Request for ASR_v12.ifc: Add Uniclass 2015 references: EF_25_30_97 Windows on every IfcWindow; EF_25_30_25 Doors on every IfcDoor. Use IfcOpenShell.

First a look at what the model holds.

```python
import ifcopenshell

model = ifcopenshell.open("ASR_v12.ifc")
print(model.schema)
print("classifications:", [c.Name for c in model.by_type("IfcClassification")])
for ifc_class in ("IfcDoor", "IfcRoof", "IfcStair", "IfcWall", "IfcWindow"):
    print(ifc_class, len(model.by_type(ifc_class)))
```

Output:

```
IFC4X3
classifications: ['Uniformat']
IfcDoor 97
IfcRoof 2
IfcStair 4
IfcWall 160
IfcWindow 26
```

```python
import ifcopenshell
import ifcopenshell.api.classification

model = ifcopenshell.open("ASR_v12.ifc")

system = ifcopenshell.api.classification.add_classification(model, classification="Uniclass 2015")

codes = {
    "IfcWindow": ("EF_25_30_97", "Windows"),
    "IfcDoor": ("EF_25_30_25", "Doors"),
}
for ifc_class, (code, name) in codes.items():
    products = model.by_type(ifc_class)
    ifcopenshell.api.classification.add_reference(
        model, products=products, classification=system, identification=code, name=name
    )
    print(code, len(products))

model.write("ASR_v12-out.ifc")
```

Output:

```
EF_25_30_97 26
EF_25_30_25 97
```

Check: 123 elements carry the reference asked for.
